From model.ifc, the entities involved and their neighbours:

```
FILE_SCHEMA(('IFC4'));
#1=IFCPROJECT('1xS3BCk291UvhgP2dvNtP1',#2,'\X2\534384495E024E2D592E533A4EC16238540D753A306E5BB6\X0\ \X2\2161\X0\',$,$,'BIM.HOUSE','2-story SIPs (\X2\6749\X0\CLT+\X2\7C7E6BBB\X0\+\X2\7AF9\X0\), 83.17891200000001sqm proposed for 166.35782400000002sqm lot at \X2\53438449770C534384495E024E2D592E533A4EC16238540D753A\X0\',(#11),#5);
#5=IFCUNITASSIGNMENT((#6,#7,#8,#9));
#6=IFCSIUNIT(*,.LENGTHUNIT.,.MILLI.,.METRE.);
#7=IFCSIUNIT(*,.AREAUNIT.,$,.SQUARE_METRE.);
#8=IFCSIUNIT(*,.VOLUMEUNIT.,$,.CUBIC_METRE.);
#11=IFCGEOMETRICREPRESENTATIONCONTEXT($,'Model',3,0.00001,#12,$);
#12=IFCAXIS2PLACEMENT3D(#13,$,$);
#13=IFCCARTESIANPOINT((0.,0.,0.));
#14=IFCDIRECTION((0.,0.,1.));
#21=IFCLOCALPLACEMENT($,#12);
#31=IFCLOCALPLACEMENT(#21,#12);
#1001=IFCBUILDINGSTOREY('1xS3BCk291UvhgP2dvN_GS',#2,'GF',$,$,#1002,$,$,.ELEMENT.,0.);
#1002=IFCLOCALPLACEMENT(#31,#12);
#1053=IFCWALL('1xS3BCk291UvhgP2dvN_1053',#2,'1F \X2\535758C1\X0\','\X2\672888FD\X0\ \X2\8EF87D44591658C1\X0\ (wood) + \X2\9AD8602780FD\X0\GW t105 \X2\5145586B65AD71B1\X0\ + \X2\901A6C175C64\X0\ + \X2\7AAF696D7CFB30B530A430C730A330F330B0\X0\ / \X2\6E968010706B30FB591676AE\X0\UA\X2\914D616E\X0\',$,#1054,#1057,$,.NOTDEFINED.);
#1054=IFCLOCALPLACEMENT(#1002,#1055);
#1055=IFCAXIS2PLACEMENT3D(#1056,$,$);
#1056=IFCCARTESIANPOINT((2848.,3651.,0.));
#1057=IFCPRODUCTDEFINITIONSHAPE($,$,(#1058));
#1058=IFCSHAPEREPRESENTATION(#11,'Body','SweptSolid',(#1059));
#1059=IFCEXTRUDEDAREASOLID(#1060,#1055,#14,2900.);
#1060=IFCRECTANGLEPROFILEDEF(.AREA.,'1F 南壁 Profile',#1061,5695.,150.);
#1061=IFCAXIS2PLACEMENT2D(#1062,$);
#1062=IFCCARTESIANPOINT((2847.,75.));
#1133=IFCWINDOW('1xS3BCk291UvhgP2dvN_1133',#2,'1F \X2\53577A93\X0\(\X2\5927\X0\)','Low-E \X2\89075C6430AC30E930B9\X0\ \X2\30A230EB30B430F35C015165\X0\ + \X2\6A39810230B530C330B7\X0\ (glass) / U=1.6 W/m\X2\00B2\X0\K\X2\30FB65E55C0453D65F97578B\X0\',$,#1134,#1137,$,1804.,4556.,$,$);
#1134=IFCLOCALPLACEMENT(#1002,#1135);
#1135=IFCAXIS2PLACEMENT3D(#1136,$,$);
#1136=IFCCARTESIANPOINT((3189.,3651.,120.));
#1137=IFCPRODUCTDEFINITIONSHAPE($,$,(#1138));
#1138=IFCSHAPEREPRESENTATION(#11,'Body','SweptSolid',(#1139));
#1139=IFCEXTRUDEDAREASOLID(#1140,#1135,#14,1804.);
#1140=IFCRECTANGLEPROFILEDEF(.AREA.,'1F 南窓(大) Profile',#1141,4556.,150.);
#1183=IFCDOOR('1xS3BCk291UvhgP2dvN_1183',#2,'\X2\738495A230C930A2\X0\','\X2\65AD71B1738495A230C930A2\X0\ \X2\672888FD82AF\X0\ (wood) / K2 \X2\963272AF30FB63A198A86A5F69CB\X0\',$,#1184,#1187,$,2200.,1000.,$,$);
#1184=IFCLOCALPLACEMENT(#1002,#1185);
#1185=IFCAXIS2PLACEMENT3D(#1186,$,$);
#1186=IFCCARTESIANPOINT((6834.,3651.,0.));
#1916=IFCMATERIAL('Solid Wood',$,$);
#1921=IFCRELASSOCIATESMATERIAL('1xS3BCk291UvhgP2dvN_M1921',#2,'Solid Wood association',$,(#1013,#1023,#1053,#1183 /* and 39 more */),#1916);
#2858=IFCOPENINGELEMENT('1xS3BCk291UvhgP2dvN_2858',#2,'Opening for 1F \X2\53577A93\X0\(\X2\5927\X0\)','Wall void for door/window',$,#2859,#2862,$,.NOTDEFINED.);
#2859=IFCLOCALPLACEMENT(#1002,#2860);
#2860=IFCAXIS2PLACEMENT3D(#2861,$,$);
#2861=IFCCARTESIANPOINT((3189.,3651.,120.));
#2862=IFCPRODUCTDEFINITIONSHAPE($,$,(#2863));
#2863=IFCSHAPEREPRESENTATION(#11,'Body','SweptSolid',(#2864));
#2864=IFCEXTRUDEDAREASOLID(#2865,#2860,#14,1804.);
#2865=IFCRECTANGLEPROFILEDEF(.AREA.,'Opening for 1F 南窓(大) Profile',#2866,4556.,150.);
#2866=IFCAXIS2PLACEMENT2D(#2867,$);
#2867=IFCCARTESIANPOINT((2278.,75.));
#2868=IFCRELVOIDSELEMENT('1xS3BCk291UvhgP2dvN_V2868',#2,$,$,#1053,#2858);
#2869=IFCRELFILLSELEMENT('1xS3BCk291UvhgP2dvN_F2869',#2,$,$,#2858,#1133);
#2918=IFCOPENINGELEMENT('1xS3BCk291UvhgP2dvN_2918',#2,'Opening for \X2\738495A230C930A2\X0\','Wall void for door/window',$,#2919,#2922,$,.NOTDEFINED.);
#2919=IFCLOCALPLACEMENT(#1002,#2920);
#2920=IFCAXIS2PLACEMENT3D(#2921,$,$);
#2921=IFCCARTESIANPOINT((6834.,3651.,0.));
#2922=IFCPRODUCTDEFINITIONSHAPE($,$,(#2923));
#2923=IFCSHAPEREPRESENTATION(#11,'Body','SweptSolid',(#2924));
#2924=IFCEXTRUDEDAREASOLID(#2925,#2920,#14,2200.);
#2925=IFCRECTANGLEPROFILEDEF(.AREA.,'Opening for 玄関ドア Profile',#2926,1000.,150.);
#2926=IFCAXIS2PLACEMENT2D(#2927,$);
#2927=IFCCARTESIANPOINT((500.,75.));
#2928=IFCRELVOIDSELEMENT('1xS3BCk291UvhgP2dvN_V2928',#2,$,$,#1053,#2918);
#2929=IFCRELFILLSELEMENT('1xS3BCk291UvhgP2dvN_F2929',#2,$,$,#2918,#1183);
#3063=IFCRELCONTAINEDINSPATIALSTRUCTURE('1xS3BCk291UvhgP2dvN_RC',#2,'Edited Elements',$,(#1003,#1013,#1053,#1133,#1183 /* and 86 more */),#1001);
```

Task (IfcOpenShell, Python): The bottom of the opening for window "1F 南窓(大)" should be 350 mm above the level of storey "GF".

```python
import numpy as np
import ifcopenshell
import ifcopenshell.api.geometry
import ifcopenshell.geom
import ifcopenshell.util.element
import ifcopenshell.util.placement
import ifcopenshell.util.shape
import ifcopenshell.util.unit

model = ifcopenshell.open("model.ifc")
unit_scale = ifcopenshell.util.unit.calculate_unit_scale(model)

window = model.by_id(1133)
opening = window.FillsVoids[0].RelatingOpeningElement
storey = ifcopenshell.util.element.get_container(window, ifc_class="IfcBuildingStorey")
level = ifcopenshell.util.placement.get_local_placement(storey.ObjectPlacement)[2, 3]

# The opening's origin need not be at the sill, so measure its lowest point.
shape = ifcopenshell.geom.create_shape(ifcopenshell.geom.settings(), opening)
bottom = ifcopenshell.util.shape.get_shape_bottom_elevation(shape, shape.geometry) / unit_scale
dz = level + 0.35 / unit_scale - bottom

shift = np.array([0.0, 0.0, dz])
# The window is not placed relative to its opening, so move both.
for product in (opening, window):
    matrix = ifcopenshell.util.placement.get_local_placement(product.ObjectPlacement)
    matrix[:3, 3] += shift
    ifcopenshell.api.geometry.edit_object_placement(model, product=product, matrix=matrix, is_si=False)

print(f"moved by {dz * unit_scale:+.3f} m")

model.write("model_v2.ifc")
```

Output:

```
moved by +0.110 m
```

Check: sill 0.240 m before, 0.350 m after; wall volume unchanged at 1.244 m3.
